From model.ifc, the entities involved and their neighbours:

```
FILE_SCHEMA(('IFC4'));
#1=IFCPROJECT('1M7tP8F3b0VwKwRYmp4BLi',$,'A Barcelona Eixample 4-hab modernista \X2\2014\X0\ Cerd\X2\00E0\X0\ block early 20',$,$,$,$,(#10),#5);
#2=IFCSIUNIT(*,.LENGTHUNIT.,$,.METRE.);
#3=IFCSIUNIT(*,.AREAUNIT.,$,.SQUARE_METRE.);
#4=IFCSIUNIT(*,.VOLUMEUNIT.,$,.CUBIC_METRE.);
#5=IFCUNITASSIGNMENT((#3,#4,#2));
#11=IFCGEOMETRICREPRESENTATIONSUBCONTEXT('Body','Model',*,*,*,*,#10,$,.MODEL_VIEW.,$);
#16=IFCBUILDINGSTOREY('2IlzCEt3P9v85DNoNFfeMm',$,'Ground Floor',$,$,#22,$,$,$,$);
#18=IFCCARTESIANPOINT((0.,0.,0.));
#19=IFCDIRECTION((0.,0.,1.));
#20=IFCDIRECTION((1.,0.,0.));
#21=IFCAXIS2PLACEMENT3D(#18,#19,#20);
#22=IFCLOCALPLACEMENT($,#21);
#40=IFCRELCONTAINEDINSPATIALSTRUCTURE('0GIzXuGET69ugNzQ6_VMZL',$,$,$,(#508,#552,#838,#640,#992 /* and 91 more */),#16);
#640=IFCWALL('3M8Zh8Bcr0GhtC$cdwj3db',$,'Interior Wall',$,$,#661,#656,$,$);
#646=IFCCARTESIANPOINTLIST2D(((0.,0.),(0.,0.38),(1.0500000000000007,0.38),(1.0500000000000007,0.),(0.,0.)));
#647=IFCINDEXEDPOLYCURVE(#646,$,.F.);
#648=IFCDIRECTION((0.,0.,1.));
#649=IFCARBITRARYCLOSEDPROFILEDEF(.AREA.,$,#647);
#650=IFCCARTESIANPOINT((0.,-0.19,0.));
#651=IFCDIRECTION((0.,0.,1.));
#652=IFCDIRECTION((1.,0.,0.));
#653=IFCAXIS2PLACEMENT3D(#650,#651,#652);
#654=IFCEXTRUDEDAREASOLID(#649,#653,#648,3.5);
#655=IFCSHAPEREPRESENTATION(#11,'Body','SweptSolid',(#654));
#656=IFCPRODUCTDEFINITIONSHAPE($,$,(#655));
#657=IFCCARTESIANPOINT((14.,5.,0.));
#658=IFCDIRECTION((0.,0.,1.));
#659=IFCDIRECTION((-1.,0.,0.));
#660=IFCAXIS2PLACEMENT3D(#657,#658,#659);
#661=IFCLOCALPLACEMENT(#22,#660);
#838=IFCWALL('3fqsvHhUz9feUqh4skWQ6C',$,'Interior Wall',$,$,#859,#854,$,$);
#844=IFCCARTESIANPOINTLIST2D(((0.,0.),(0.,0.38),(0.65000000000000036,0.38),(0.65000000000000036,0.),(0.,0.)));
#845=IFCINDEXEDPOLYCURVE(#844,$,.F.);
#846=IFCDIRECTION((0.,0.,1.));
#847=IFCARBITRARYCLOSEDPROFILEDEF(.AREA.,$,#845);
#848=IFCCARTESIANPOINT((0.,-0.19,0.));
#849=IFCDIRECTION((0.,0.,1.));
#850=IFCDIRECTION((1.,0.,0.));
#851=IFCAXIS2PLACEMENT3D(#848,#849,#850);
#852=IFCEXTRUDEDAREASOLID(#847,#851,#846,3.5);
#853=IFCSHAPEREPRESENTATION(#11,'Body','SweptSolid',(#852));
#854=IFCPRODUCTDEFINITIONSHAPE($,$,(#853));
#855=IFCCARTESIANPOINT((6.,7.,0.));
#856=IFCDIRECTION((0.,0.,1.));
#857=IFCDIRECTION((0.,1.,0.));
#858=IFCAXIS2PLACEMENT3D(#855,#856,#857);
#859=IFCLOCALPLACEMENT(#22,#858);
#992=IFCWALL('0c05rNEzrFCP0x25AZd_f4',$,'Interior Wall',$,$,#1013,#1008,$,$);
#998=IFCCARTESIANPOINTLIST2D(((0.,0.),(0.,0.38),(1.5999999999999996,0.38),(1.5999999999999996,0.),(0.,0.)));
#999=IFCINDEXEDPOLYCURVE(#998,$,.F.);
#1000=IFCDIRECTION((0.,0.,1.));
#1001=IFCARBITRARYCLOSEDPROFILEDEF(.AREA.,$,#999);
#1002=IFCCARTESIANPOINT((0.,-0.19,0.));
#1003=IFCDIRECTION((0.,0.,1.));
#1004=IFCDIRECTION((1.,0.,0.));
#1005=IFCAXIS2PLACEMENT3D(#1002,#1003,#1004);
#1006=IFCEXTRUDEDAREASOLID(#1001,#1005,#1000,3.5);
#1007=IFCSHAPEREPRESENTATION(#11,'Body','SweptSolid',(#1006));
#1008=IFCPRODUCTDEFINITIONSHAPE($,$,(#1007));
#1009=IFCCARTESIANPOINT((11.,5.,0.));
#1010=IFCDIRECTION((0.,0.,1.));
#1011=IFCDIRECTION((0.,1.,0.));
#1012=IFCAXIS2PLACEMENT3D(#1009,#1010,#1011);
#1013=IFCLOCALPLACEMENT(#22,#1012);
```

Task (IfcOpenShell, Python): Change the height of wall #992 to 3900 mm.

```python
import ifcopenshell
import ifcopenshell.geom
import ifcopenshell.util.representation
import ifcopenshell.util.shape

model = ifcopenshell.open("model.ifc")
settings = ifcopenshell.geom.settings()


def volume(element):
    """Net volume in cubic metres, openings subtracted."""
    shape = ifcopenshell.geom.create_shape(settings, element)
    return ifcopenshell.util.shape.get_volume(shape.geometry)


wall = model.by_guid("0c05rNEzrFCP0x25AZd_f4")
before = volume(wall)

body = ifcopenshell.util.representation.get_representation(wall, "Model", "Body")
solid = body.Items[0]
old_height = solid.Depth
solid.Depth = 3.9
after = volume(wall)

print(f"height {old_height:g} -> {solid.Depth:g}, volume {before:.3f} -> {after:.3f} m3")

model.write("model-out.ifc")
```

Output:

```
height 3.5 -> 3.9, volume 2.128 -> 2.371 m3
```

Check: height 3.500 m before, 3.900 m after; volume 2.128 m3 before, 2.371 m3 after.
